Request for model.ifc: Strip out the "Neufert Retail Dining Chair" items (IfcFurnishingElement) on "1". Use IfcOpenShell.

First a look at what the model holds.

```python
import ifcopenshell
import ifcopenshell.util.element

model = ifcopenshell.open("model.ifc")
print(model.schema)
storey = next(s for s in model.by_type("IfcBuildingStorey") if s.Name == "1")
furniture = [e for e in ifcopenshell.util.element.get_decomposition(storey) if e.is_a("IfcFurnishingElement")]
seen = {}
for e in furniture:
    element_type = ifcopenshell.util.element.get_type(e)
    name = element_type.Name if element_type not in (None, e) else None
    seen[name] = seen.get(name, 0) + 1
for name, count in sorted(seen.items(), key=str):
    print(count, "x", name)
```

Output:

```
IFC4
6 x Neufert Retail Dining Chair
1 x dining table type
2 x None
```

```python
import ifcopenshell
import ifcopenshell.api.root
import ifcopenshell.util.element

model = ifcopenshell.open("model.ifc")

storey = next(s for s in model.by_type("IfcBuildingStorey") if s.Name == "1")
furniture = [e for e in ifcopenshell.util.element.get_decomposition(storey) if e.is_a("IfcFurnishingElement")]
targets = [e for e in furniture if (t := ifcopenshell.util.element.get_type(e)) not in (None, e) and t.Name == "Neufert Retail Dining Chair"]

for e in targets:
    ifcopenshell.api.root.remove_product(model, product=e)
print(len(targets), "removed")

model.write("model_rev.ifc")
```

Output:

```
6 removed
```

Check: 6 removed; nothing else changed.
